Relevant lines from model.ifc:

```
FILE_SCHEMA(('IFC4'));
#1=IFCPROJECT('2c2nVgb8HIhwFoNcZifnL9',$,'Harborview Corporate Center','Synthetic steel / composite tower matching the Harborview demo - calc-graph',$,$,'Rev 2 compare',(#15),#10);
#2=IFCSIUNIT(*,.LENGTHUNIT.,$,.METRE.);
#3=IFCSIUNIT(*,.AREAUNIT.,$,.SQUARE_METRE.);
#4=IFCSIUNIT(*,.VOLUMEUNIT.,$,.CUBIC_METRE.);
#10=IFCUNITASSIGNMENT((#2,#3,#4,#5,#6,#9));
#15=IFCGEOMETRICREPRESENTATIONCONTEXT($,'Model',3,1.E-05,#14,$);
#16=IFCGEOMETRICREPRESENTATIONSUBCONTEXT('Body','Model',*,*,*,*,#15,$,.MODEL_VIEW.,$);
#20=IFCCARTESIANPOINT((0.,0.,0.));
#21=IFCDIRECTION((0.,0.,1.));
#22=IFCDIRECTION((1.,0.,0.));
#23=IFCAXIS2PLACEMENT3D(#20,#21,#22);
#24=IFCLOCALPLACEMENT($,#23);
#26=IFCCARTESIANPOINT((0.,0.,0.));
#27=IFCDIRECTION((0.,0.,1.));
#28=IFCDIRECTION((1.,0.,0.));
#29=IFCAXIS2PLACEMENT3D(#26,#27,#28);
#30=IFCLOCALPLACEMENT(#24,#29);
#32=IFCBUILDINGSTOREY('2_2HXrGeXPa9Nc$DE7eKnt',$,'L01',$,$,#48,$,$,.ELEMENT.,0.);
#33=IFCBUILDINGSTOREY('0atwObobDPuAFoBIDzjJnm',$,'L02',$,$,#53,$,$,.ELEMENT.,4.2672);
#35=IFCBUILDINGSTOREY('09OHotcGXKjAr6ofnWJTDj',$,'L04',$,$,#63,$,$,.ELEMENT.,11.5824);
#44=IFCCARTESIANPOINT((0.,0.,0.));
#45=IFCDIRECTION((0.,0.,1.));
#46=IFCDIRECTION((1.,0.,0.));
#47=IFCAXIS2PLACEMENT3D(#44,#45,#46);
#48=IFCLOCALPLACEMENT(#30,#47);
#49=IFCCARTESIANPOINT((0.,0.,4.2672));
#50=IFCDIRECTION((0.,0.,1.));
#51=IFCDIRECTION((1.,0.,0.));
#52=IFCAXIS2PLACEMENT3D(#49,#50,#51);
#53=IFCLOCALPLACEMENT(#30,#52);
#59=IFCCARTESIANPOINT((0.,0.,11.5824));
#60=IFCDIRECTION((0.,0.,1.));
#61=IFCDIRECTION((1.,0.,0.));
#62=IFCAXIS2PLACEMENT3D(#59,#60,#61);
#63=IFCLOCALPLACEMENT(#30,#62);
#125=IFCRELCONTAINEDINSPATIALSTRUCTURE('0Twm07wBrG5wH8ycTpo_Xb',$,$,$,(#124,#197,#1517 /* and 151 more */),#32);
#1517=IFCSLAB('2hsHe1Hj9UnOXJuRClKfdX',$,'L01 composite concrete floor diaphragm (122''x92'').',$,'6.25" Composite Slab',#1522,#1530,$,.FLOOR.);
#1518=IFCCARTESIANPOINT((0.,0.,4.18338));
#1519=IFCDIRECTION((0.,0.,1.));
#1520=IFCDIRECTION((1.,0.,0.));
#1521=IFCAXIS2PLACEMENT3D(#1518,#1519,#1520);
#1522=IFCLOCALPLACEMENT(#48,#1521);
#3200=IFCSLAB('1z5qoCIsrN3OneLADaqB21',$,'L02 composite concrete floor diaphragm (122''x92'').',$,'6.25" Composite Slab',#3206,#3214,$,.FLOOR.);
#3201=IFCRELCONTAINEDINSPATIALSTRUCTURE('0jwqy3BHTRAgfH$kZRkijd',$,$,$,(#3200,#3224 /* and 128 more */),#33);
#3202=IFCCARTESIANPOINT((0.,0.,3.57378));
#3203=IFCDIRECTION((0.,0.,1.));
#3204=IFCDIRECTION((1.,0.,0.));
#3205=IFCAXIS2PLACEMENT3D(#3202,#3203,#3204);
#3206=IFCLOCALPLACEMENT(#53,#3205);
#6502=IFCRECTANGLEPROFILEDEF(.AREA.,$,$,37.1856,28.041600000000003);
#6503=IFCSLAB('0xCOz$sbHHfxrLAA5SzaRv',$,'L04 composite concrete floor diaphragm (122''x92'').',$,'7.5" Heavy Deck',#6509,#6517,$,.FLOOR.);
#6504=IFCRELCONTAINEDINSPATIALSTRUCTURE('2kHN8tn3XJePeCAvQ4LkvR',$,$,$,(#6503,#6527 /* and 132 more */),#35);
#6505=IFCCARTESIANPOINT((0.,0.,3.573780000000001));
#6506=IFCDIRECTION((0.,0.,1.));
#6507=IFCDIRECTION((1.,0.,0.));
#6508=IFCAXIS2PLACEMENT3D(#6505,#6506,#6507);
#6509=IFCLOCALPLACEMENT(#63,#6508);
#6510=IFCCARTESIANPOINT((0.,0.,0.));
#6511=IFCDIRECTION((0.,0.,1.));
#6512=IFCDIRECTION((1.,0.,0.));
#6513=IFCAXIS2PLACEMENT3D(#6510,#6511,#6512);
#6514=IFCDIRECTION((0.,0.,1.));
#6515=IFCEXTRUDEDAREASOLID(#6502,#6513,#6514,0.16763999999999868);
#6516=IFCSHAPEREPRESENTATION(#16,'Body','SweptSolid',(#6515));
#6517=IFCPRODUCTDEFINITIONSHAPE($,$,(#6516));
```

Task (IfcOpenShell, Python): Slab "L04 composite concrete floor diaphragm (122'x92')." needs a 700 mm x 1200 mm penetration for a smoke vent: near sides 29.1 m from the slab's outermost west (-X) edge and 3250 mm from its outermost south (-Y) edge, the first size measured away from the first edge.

```python
import numpy as np
import ifcopenshell
import ifcopenshell.api.feature
import ifcopenshell.api.geometry
import ifcopenshell.api.root
import ifcopenshell.geom
import ifcopenshell.util.placement
import ifcopenshell.util.representation
import ifcopenshell.util.shape
import ifcopenshell.util.unit

model = ifcopenshell.open("model.ifc")
unit_scale = ifcopenshell.util.unit.calculate_unit_scale(model)
settings = ifcopenshell.geom.settings()


def volume(element):
    """Net volume in cubic metres, openings subtracted."""
    shape = ifcopenshell.geom.create_shape(settings, element)
    return ifcopenshell.util.shape.get_volume(shape.geometry)


slab = model.by_id(6503)
before = volume(slab)

# Extent in the slab's own axes, in metres. The edges named are its -X and -Y sides.
slab_shape = ifcopenshell.geom.create_shape(settings, slab)
vertices = ifcopenshell.util.shape.get_vertices(slab_shape.geometry)
x_min, y_min, bottom = vertices.min(axis=0)
top = vertices[:, 2].max()

opening = ifcopenshell.api.root.create_entity(model, ifc_class="IfcOpeningElement", name="Smoke vent opening", predefined_type="OPENING")
context = ifcopenshell.util.representation.get_context(model, "Model", "Body", "MODEL_VIEW")
width, depth = 0.7, 1.2
outline = [(0.0, 0.0), (width, 0.0), (width, depth), (0.0, depth), (0.0, 0.0)]
# Overshoot both faces by 50 mm so the cut is clean.
shape = ifcopenshell.api.geometry.add_slab_representation(
    model, context=context, depth=top - bottom + 0.1, polyline=outline
)
ifcopenshell.api.geometry.assign_representation(model, product=opening, representation=shape)

matrix = ifcopenshell.util.placement.get_local_placement(slab.ObjectPlacement)
matrix[:, 3] = matrix @ np.append(np.array([x_min + 29.1, y_min + 3.25, bottom - 0.05]) / unit_scale, 1.0)
ifcopenshell.api.geometry.edit_object_placement(model, product=opening, matrix=matrix, is_si=False)
ifcopenshell.api.feature.add_feature(model, feature=opening, element=slab)

after = volume(slab)

print(f"slab volume {before:.3f} -> {after:.3f} m3")

model.write("model_updated.ifc")
```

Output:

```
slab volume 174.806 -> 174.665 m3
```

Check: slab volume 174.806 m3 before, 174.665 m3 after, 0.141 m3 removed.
